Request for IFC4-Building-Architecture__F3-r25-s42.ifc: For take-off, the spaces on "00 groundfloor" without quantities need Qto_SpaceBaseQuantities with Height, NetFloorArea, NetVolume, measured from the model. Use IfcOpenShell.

First a look at what the model holds.

```python
import ifcopenshell
import ifcopenshell.util.element
import ifcopenshell.util.unit

model = ifcopenshell.open("IFC4-Building-Architecture__F3-r25-s42.ifc")
print(model.schema)
for unit_type in ("LENGTHUNIT", "AREAUNIT", "VOLUMEUNIT"):
    print(unit_type, ifcopenshell.util.unit.calculate_unit_scale(model, unit_type))
storey = next(s for s in model.by_type("IfcBuildingStorey") if s.Name == "00 groundfloor")
spaces = [e for e in ifcopenshell.util.element.get_decomposition(storey) if e.is_a("IfcSpace")]
for e in sorted(spaces, key=lambda e: e.id()):
    print(e.id(), e.is_a(), e.Name, list(ifcopenshell.util.element.get_psets(e, qtos_only=True)), sep=" | ")
```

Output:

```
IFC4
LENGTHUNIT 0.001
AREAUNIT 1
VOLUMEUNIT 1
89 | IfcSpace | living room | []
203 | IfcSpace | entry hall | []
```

```python
import ifcopenshell
import ifcopenshell.api.pset
import ifcopenshell.geom
import ifcopenshell.util.element
import ifcopenshell.util.shape
import ifcopenshell.util.unit

model = ifcopenshell.open("IFC4-Building-Architecture__F3-r25-s42.ifc")
unit_scale = ifcopenshell.util.unit.calculate_unit_scale(model)
area_scale = ifcopenshell.util.unit.calculate_unit_scale(model, "AREAUNIT")
volume_scale = ifcopenshell.util.unit.calculate_unit_scale(model, "VOLUMEUNIT")
settings = ifcopenshell.geom.settings()

storey = next(s for s in model.by_type("IfcBuildingStorey") if s.Name == "00 groundfloor")
spaces = [e for e in ifcopenshell.util.element.get_decomposition(storey) if e.is_a("IfcSpace")]

for e in sorted(spaces, key=lambda e: e.id()):
    if ifcopenshell.util.element.get_psets(e, qtos_only=True, should_inherit=False):
        continue
    # Geometry comes back in metres, in the element's own axes.
    shape = ifcopenshell.geom.create_shape(settings, e)
    values = {
        "Height": ifcopenshell.util.shape.get_z(shape.geometry) / unit_scale,
        "NetFloorArea": ifcopenshell.util.shape.get_footprint_area(shape.geometry) / area_scale,
        "NetVolume": ifcopenshell.util.shape.get_volume(shape.geometry) / volume_scale,
    }
    qto = ifcopenshell.api.pset.add_qto(model, product=e, name="Qto_SpaceBaseQuantities")
    ifcopenshell.api.pset.edit_qto(model, qto=qto, properties=values)
    print(e.id(), {k: round(v, 3) for k, v in values.items()})

model.write("IFC4-Building-Architecture__F3-r25-s42_updated.ifc")
```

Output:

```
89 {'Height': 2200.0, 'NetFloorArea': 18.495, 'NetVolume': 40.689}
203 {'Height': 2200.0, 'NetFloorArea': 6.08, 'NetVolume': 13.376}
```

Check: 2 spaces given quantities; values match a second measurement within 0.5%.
